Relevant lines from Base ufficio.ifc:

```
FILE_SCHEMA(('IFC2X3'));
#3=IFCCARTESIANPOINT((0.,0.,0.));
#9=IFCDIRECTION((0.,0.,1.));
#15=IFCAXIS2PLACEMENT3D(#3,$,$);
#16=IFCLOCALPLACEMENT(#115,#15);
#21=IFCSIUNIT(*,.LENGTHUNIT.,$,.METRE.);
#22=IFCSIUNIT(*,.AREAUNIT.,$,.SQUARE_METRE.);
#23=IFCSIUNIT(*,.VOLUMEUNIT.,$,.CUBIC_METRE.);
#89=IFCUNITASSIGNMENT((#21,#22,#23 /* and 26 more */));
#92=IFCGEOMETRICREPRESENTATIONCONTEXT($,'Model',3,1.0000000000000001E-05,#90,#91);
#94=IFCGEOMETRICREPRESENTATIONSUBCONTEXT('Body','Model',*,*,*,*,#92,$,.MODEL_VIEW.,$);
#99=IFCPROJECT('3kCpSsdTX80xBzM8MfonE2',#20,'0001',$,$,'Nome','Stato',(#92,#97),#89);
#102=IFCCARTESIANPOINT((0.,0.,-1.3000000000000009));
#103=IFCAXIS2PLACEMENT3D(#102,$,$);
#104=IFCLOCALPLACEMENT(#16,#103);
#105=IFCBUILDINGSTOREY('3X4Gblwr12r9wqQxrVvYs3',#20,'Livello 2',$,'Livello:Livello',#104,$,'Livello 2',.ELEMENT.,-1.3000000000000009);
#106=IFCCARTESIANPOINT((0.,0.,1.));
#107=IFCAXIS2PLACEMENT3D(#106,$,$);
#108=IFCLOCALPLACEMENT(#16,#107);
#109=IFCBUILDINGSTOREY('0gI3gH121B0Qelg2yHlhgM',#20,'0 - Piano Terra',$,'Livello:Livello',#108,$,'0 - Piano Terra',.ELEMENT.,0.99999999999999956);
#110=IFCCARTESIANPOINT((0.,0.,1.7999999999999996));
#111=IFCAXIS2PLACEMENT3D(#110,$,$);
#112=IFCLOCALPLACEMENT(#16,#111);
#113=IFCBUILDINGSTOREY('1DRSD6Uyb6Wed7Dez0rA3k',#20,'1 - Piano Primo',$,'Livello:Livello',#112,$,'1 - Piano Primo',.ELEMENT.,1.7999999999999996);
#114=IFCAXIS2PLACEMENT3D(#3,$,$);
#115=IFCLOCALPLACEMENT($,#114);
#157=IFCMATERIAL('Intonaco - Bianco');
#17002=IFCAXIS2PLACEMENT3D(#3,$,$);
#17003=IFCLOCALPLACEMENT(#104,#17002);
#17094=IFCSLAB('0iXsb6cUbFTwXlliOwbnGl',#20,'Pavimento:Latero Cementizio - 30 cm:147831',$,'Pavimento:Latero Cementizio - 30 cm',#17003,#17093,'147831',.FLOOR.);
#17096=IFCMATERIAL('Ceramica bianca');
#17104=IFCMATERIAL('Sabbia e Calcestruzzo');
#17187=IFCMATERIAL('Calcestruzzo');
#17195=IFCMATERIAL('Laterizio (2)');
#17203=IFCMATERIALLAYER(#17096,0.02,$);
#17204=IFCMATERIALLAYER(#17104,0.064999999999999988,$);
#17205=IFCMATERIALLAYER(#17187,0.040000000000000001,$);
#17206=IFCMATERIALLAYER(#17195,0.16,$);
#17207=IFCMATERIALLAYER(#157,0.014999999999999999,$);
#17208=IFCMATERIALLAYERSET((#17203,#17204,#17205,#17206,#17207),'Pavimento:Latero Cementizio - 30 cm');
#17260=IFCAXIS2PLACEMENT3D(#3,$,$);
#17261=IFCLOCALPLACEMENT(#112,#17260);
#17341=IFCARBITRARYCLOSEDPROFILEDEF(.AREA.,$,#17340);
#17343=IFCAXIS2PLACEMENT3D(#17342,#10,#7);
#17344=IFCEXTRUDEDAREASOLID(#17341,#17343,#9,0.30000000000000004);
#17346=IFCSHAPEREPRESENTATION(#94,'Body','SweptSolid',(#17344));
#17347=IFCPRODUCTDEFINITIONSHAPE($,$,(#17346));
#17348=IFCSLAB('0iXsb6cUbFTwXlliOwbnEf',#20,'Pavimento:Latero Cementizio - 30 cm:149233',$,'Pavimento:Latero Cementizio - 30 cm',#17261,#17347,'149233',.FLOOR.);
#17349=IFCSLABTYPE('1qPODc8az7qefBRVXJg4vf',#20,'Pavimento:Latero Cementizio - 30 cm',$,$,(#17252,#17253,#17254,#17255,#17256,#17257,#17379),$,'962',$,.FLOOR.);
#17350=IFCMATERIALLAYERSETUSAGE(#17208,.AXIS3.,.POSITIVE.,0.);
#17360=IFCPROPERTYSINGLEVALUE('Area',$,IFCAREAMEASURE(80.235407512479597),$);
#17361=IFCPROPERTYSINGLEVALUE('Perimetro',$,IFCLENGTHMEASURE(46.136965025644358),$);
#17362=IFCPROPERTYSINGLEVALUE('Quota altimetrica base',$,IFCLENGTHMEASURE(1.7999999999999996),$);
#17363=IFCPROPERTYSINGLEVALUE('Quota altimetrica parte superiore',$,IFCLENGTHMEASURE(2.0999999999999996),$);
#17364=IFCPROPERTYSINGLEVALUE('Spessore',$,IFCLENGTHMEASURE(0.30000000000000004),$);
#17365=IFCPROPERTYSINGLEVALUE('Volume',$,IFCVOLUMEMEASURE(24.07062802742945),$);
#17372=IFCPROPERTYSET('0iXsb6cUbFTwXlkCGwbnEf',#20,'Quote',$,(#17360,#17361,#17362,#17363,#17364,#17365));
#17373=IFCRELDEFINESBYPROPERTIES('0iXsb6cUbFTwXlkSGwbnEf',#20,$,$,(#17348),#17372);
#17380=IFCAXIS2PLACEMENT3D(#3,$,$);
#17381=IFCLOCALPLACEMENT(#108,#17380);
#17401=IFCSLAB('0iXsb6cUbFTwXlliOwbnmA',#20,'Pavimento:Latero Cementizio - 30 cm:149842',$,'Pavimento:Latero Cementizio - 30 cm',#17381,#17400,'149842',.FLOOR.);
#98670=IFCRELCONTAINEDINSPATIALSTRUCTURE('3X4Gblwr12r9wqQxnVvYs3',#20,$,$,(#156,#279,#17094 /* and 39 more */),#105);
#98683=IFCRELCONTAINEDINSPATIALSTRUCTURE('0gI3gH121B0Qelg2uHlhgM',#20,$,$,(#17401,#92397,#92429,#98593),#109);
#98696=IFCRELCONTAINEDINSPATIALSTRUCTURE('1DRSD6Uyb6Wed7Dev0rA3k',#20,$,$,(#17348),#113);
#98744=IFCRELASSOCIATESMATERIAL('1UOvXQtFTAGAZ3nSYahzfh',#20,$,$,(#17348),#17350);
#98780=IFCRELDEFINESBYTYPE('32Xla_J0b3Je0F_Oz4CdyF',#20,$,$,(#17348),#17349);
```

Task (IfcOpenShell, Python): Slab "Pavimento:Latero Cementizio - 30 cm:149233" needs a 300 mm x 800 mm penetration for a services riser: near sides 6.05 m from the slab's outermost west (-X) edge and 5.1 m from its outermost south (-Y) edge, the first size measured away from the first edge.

```python
import numpy as np
import ifcopenshell
import ifcopenshell.api.feature
import ifcopenshell.api.geometry
import ifcopenshell.api.pset
import ifcopenshell.api.root
import ifcopenshell.geom
import ifcopenshell.util.element
import ifcopenshell.util.placement
import ifcopenshell.util.representation
import ifcopenshell.util.shape
import ifcopenshell.util.unit

model = ifcopenshell.open("Base ufficio.ifc")
unit_scale = ifcopenshell.util.unit.calculate_unit_scale(model)
area_scale = ifcopenshell.util.unit.calculate_unit_scale(model, "AREAUNIT")
volume_scale = ifcopenshell.util.unit.calculate_unit_scale(model, "VOLUMEUNIT")
settings = ifcopenshell.geom.settings()


def volume(element):
    """Net volume in cubic metres, openings subtracted."""
    shape = ifcopenshell.geom.create_shape(settings, element)
    return ifcopenshell.util.shape.get_volume(shape.geometry)


slab = model.by_id(17348)
before = volume(slab)

# Extent in the slab's own axes, in metres. The edges named are its -X and -Y sides.
slab_shape = ifcopenshell.geom.create_shape(settings, slab)
vertices = ifcopenshell.util.shape.get_vertices(slab_shape.geometry)
x_min, y_min, bottom = vertices.min(axis=0)
top = vertices[:, 2].max()

opening = ifcopenshell.api.root.create_entity(model, ifc_class="IfcOpeningElement", name="Services riser opening")
context = ifcopenshell.util.representation.get_context(model, "Model", "Body", "MODEL_VIEW")
width, depth = 0.3, 0.8
outline = [(0.0, 0.0), (width, 0.0), (width, depth), (0.0, depth), (0.0, 0.0)]
# Overshoot both faces by 50 mm so the cut is clean.
shape = ifcopenshell.api.geometry.add_slab_representation(
    model, context=context, depth=top - bottom + 0.1, polyline=outline
)
ifcopenshell.api.geometry.assign_representation(model, product=opening, representation=shape)

matrix = ifcopenshell.util.placement.get_local_placement(slab.ObjectPlacement)
matrix[:, 3] = matrix @ np.append(np.array([x_min + 6.05, y_min + 5.1, bottom - 0.05]) / unit_scale, 1.0)
ifcopenshell.api.geometry.edit_object_placement(model, product=opening, matrix=matrix, is_si=False)
ifcopenshell.api.feature.add_feature(model, feature=opening, element=slab)

after = volume(slab)

# Update the slab's stored quantities.
pset = model.by_id(ifcopenshell.util.element.get_pset(slab, "Quote", should_inherit=False)["id"])
ifcopenshell.api.pset.edit_pset(model, pset=pset, properties={
    "Area": model.create_entity("IfcAreaMeasure", after / (top - bottom) / area_scale),
    "Volume": model.create_entity("IfcVolumeMeasure", after / volume_scale),
})

print(f"slab volume {before:.3f} -> {after:.3f} m3")

model.write("Base ufficio_v2.ifc")
```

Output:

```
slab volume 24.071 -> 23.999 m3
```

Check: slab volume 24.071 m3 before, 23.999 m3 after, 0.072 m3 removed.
